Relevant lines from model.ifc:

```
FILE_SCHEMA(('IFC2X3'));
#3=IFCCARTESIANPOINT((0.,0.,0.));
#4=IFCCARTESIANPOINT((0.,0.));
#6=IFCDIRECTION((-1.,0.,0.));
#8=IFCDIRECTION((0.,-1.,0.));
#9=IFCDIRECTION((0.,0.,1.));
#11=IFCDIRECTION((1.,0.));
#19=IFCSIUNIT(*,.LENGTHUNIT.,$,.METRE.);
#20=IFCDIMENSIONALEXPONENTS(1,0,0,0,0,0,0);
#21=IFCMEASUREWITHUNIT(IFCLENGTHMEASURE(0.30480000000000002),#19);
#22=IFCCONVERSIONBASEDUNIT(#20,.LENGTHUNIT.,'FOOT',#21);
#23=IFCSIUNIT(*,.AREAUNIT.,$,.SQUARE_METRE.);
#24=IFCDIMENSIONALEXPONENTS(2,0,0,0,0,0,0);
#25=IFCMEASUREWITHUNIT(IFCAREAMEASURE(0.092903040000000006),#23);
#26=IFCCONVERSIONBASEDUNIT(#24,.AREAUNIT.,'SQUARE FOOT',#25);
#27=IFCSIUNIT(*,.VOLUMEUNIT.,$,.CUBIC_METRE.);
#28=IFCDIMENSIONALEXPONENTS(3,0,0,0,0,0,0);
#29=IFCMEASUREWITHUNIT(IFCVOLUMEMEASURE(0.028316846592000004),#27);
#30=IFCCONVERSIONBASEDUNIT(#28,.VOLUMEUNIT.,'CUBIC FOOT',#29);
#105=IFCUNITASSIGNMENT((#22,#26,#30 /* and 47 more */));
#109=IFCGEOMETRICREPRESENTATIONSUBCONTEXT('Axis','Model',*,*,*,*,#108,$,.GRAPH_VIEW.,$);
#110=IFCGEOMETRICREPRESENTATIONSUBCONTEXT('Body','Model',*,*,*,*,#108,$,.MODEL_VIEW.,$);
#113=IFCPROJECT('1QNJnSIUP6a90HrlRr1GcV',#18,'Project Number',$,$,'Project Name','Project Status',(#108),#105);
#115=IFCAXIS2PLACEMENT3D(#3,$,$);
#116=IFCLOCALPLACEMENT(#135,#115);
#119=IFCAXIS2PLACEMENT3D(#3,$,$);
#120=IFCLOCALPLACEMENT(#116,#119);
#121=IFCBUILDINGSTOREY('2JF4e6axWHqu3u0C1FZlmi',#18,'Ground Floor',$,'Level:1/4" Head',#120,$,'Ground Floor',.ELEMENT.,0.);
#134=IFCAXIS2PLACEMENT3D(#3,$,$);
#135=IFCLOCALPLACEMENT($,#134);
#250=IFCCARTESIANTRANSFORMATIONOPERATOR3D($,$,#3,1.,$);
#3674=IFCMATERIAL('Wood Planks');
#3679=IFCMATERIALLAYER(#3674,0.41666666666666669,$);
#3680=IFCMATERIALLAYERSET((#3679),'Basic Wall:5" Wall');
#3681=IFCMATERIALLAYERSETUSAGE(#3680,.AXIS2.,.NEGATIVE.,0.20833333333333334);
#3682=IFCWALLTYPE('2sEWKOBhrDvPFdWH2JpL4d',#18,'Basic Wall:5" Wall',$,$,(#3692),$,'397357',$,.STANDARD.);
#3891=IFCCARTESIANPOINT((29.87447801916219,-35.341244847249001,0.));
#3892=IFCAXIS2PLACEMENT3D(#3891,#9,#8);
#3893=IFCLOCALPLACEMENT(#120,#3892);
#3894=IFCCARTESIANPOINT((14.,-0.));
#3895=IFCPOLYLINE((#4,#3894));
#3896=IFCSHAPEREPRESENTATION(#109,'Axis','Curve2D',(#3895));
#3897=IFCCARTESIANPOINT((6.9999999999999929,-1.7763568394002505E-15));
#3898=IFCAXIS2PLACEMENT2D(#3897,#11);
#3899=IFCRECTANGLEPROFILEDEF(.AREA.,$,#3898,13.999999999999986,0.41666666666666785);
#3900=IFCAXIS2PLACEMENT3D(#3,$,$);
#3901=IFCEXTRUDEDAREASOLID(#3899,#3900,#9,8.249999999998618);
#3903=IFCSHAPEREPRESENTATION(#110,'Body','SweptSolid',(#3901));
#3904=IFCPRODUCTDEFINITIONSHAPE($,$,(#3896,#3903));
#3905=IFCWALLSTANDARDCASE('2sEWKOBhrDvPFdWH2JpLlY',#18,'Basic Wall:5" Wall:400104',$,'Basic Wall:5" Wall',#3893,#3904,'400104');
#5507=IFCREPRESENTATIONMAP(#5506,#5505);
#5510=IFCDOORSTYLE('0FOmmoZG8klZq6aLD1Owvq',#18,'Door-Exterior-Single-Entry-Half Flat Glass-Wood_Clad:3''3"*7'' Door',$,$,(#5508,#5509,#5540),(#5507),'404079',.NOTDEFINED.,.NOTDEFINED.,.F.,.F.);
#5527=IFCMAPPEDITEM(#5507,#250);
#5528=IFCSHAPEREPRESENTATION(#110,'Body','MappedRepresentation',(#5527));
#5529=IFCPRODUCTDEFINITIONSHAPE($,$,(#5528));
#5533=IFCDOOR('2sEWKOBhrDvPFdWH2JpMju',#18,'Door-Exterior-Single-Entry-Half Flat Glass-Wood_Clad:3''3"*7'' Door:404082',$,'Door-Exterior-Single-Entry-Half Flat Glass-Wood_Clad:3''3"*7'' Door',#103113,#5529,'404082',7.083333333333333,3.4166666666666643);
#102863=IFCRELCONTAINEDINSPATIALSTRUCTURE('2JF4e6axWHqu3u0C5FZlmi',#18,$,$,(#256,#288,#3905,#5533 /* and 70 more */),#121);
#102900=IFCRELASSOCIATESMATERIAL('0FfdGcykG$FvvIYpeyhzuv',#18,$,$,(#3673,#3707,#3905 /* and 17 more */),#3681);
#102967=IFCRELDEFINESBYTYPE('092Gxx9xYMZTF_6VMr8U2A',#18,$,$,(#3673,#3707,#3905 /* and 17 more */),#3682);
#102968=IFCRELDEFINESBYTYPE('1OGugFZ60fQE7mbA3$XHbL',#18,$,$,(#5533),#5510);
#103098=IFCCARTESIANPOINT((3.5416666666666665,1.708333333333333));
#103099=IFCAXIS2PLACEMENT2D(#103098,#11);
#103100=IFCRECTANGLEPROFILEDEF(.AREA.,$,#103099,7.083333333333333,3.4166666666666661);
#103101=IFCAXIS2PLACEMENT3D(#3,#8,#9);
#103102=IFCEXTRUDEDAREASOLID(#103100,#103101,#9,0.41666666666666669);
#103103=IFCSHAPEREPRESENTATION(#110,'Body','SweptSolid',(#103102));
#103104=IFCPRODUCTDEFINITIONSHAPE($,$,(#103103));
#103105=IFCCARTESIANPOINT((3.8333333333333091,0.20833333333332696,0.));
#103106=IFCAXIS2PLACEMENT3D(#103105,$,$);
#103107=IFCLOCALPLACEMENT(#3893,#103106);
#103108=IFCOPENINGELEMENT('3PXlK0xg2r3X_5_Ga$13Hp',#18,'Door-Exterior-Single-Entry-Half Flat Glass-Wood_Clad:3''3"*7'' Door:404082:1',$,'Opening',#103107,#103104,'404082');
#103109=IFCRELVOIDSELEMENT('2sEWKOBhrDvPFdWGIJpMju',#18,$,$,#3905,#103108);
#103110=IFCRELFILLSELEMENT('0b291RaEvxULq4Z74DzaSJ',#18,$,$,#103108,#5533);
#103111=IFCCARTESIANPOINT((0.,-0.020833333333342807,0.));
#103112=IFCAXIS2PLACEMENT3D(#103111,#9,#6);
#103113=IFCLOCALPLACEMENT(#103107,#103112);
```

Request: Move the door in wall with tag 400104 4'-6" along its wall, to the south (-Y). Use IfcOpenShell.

```python
import ifcopenshell
import ifcopenshell.api.geometry
import ifcopenshell.util.placement
import ifcopenshell.util.unit

model = ifcopenshell.open("model.ifc")
unit_scale = ifcopenshell.util.unit.calculate_unit_scale(model)

door = model.by_guid("2sEWKOBhrDvPFdWH2JpMju")
opening = door.FillsVoids[0].RelatingOpeningElement
wall = opening.VoidsElements[0].RelatingBuildingElement

wall_matrix = ifcopenshell.util.placement.get_local_placement(wall.ObjectPlacement)
shift = wall_matrix[:3, 0] * 54 * 0.0254 / unit_scale
before = ifcopenshell.util.placement.get_local_placement(door.ObjectPlacement)[:3, 3].copy()

# The door is placed relative to its opening, so it follows when the opening moves.
matrix = ifcopenshell.util.placement.get_local_placement(opening.ObjectPlacement)
matrix[:3, 3] += shift
ifcopenshell.api.geometry.edit_object_placement(
    model, product=opening, matrix=matrix, is_si=False, should_transform_children=True
)

after = ifcopenshell.util.placement.get_local_placement(door.ObjectPlacement)[:3, 3]
print("door moved by", (after - before).round(3) + 0.0)

model.write("model_v2.ifc")
```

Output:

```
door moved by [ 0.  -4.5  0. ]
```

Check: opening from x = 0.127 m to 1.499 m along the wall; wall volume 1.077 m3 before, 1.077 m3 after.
